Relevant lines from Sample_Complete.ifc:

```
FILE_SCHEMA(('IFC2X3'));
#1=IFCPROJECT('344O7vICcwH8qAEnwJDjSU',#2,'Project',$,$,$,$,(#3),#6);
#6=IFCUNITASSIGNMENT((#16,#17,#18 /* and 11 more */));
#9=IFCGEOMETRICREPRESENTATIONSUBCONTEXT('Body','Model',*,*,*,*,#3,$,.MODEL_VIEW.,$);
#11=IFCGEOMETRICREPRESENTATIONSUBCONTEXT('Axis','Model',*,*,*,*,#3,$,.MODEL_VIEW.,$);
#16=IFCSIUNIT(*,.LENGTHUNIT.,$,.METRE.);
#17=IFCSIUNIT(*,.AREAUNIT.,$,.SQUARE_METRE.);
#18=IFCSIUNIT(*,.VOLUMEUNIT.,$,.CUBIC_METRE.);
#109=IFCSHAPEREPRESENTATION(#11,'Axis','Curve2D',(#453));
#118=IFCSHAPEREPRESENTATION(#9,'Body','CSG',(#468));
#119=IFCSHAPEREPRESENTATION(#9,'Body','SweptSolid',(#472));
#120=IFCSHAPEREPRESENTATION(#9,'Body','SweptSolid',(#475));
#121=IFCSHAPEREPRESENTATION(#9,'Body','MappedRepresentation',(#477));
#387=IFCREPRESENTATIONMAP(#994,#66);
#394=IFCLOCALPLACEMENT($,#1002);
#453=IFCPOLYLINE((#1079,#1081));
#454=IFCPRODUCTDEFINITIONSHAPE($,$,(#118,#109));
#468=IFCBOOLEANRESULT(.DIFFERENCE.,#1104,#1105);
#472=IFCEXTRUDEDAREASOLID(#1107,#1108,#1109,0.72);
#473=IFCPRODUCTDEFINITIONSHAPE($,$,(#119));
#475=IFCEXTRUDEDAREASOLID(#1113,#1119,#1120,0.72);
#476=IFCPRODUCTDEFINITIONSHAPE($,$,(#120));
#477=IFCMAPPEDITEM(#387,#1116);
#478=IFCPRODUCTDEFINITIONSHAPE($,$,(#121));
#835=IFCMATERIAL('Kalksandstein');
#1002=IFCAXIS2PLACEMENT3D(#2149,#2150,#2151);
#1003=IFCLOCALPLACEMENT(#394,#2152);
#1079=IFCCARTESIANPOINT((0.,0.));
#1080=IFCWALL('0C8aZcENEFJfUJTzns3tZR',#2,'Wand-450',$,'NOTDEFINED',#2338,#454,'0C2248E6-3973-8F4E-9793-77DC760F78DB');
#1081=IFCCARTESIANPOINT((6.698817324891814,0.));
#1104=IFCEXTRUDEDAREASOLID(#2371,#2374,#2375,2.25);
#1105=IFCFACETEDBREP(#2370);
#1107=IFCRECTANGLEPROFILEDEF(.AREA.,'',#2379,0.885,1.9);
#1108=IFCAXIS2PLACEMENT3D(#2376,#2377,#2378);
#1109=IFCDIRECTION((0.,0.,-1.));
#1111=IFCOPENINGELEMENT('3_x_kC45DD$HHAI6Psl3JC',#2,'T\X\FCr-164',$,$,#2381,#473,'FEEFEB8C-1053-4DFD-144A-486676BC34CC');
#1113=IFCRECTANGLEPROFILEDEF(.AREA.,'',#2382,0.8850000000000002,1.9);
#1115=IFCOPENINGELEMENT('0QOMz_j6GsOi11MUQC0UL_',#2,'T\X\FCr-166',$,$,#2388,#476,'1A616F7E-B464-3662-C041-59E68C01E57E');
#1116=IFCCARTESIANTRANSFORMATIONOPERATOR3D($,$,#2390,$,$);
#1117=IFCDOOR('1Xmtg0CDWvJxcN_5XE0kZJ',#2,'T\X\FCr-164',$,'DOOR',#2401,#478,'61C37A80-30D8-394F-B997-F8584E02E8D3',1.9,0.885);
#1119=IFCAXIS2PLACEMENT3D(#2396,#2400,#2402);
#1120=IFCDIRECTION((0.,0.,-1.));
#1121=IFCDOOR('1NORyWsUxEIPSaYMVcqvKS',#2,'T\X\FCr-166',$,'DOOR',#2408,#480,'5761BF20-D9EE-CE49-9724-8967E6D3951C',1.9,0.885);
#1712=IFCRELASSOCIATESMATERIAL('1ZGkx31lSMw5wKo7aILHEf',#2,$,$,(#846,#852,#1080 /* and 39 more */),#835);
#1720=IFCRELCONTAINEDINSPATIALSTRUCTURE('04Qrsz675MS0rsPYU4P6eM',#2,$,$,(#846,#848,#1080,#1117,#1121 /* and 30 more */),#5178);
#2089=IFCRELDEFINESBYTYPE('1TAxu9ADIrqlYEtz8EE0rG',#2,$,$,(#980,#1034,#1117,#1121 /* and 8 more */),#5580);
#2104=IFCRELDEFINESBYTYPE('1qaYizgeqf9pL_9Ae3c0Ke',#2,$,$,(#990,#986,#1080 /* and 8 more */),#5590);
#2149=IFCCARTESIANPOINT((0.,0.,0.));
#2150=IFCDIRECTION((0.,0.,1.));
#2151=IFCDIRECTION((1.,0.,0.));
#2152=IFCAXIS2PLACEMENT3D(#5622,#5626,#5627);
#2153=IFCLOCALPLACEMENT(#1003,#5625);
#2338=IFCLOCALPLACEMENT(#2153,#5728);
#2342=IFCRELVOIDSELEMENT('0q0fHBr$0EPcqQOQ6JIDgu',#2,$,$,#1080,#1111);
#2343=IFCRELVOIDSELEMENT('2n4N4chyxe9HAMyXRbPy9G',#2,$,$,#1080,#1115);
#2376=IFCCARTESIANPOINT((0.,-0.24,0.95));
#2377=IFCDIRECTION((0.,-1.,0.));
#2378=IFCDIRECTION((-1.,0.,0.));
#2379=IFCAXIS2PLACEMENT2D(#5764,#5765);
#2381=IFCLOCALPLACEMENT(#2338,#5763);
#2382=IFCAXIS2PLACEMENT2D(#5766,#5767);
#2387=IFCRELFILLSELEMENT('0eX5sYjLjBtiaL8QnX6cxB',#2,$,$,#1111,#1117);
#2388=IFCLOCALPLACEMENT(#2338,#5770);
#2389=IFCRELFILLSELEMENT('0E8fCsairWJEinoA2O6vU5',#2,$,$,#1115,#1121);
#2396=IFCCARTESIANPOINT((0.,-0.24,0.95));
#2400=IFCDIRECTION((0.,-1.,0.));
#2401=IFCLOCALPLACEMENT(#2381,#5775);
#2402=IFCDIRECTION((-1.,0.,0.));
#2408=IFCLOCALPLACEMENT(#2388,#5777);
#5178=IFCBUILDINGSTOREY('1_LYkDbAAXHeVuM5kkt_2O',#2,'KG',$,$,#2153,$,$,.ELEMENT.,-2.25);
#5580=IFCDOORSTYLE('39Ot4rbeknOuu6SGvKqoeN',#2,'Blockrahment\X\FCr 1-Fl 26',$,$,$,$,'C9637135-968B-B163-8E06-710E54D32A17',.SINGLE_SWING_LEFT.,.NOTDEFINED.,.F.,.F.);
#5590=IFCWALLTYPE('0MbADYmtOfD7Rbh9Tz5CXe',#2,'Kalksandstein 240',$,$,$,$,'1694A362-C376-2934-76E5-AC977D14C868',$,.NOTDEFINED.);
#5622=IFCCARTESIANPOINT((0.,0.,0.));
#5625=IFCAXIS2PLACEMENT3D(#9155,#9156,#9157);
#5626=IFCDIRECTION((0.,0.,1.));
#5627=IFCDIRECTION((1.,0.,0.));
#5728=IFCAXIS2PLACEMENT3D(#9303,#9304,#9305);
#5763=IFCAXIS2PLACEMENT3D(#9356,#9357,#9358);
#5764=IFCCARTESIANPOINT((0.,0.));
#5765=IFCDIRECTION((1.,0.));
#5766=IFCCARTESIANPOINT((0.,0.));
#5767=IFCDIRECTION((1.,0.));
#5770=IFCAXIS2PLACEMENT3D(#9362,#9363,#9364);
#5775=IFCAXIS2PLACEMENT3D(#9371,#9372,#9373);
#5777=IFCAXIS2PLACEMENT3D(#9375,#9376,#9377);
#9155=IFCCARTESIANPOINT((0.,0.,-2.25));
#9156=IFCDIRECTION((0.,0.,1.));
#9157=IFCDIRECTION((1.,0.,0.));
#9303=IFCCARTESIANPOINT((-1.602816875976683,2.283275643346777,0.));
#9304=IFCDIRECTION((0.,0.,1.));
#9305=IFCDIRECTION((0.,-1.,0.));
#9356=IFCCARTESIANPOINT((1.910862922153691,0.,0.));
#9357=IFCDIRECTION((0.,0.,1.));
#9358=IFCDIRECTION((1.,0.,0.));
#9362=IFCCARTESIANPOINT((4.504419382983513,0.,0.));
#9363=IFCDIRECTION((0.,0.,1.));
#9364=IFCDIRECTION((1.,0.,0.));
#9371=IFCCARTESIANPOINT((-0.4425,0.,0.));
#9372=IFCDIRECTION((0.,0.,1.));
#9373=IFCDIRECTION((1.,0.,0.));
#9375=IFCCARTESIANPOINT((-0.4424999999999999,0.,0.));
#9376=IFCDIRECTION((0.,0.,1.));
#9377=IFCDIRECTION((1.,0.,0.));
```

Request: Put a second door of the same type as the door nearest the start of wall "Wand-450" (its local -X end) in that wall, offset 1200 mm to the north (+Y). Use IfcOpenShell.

```python
import ifcopenshell
import ifcopenshell.api.feature
import ifcopenshell.api.geometry
import ifcopenshell.api.root
import ifcopenshell.geom
import ifcopenshell.util.element
import ifcopenshell.util.placement
import ifcopenshell.util.shape
import ifcopenshell.util.unit

model = ifcopenshell.open("Sample_Complete.ifc")
unit_scale = ifcopenshell.util.unit.calculate_unit_scale(model)
settings = ifcopenshell.geom.settings()


def volume(element):
    """Net volume in cubic metres, openings subtracted."""
    shape = ifcopenshell.geom.create_shape(settings, element)
    return ifcopenshell.util.shape.get_volume(shape.geometry)


def reuse_history(source, copy):
    """copy_class also copies each property set's owner history, people and application; keep the originals."""
    for rel in copy.IsDefinedBy:
        if rel.is_a("IfcRelDefinesByProperties") and (history := rel.RelatingPropertyDefinition.OwnerHistory):
            rel.RelatingPropertyDefinition.OwnerHistory = source.OwnerHistory
            ifcopenshell.util.element.remove_deep2(model, history)


door = model.by_id(1117)
opening = door.FillsVoids[0].RelatingOpeningElement
wall = opening.VoidsElements[0].RelatingBuildingElement
before = volume(wall)
shift = ifcopenshell.util.placement.get_local_placement(wall.ObjectPlacement)[:3, 0] * -1.2 / unit_scale

# copy_class copies the void relationship, type, container and properties, but no geometry.
new_opening = ifcopenshell.api.root.copy_class(model, product=opening)
new_opening.Representation = ifcopenshell.util.element.copy_deep(
    model, opening.Representation, exclude=["IfcGeometricRepresentationContext", "IfcRepresentationMap"]
)
new_opening.Tag = None
new_door = ifcopenshell.api.root.copy_class(model, product=door)
new_door.Representation = ifcopenshell.util.element.copy_deep(
    model, door.Representation, exclude=["IfcGeometricRepresentationContext", "IfcRepresentationMap"]
)
new_door.Tag = None
reuse_history(door, new_door)
fills = ifcopenshell.api.feature.add_filling(model, opening=new_opening, element=new_door)
fills.OwnerHistory = new_door.OwnerHistory  # required in IFC2X3

for old, new in ((opening, new_opening), (door, new_door)):
    matrix = ifcopenshell.util.placement.get_local_placement(old.ObjectPlacement)
    matrix[:3, 3] += shift
    ifcopenshell.api.geometry.edit_object_placement(model, product=new, matrix=matrix, is_si=False)

after = volume(wall)

print(f"wall volume {before:.3f} -> {after:.3f} m3")

model.write("Sample_Complete_rev.ifc")
```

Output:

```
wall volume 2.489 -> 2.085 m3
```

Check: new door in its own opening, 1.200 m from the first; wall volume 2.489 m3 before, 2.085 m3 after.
